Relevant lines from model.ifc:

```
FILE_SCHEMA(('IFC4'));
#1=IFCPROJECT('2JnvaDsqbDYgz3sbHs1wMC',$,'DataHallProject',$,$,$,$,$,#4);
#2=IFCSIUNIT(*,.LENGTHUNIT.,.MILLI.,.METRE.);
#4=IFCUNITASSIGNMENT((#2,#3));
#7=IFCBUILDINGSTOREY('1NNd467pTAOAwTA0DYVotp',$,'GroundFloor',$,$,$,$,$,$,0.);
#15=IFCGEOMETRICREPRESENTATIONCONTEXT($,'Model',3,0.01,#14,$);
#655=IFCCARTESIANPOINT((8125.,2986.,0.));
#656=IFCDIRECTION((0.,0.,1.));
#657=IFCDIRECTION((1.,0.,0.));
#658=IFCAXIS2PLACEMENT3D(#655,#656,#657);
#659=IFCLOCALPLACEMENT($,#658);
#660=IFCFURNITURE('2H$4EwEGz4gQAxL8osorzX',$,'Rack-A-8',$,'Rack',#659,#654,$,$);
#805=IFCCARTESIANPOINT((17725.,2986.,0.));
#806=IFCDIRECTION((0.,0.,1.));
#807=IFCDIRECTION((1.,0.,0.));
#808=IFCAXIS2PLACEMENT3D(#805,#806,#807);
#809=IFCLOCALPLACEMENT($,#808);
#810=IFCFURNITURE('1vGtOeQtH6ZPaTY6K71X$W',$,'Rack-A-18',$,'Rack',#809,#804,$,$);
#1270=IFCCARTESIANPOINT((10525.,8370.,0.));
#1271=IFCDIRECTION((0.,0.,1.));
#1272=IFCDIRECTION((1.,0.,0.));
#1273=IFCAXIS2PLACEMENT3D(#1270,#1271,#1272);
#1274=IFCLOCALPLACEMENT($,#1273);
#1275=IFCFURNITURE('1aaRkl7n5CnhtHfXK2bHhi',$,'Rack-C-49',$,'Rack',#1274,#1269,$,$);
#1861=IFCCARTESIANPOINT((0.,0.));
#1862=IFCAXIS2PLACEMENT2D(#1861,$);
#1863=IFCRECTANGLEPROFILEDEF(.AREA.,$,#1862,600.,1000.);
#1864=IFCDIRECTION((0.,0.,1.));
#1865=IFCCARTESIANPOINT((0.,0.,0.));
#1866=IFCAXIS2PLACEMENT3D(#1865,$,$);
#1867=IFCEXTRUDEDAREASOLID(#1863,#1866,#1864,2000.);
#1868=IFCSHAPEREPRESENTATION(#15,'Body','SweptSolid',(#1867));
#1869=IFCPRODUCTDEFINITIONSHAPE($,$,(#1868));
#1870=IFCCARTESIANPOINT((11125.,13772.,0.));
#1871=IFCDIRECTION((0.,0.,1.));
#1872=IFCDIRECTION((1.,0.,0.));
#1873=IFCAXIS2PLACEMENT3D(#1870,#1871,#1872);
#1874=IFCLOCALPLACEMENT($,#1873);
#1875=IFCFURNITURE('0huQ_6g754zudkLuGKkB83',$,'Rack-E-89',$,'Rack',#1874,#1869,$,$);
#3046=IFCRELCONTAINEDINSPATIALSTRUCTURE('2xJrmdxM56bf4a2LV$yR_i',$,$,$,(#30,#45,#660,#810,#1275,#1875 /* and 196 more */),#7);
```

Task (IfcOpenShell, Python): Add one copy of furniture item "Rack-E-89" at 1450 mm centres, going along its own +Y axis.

```python
import ifcopenshell
import ifcopenshell.api.geometry
import ifcopenshell.api.root
import ifcopenshell.util.element
import ifcopenshell.util.placement

model = ifcopenshell.open("model.ifc")

source = model.by_guid("0huQ_6g754zudkLuGKkB83")
base = ifcopenshell.util.placement.get_local_placement(source.ObjectPlacement)
step = base[:3, 1] * 1450.0

for i in range(1, 2):
    copy = ifcopenshell.api.root.copy_class(model, product=source)
    copy.Representation = ifcopenshell.util.element.copy_deep(
        model, source.Representation, exclude=["IfcGeometricRepresentationContext", "IfcRepresentationMap"]
    )
    matrix = base.copy()
    matrix[:3, 3] += i * step
    print("added at", matrix[:3, 3].round(3) + 0.0)
    ifcopenshell.api.geometry.edit_object_placement(model, product=copy, matrix=matrix, is_si=False)

model.write("model-out.ifc")
```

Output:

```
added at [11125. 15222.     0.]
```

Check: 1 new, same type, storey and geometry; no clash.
